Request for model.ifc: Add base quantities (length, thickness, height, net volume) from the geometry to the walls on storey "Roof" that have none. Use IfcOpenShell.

First a look at what the model holds.

```python
import ifcopenshell
import ifcopenshell.util.element
import ifcopenshell.util.unit

model = ifcopenshell.open("model.ifc")
print(model.schema)
for unit_type in ("LENGTHUNIT", "AREAUNIT", "VOLUMEUNIT"):
    print(unit_type, ifcopenshell.util.unit.calculate_unit_scale(model, unit_type))
storey = next(s for s in model.by_type("IfcBuildingStorey") if s.Name == "Roof")
walls = [e for e in ifcopenshell.util.element.get_decomposition(storey) if e.is_a("IfcWall")]
for e in sorted(walls, key=lambda e: e.id()):
    print(e.id(), e.is_a(), e.Name, list(ifcopenshell.util.element.get_psets(e, qtos_only=True)), sep=" | ")
```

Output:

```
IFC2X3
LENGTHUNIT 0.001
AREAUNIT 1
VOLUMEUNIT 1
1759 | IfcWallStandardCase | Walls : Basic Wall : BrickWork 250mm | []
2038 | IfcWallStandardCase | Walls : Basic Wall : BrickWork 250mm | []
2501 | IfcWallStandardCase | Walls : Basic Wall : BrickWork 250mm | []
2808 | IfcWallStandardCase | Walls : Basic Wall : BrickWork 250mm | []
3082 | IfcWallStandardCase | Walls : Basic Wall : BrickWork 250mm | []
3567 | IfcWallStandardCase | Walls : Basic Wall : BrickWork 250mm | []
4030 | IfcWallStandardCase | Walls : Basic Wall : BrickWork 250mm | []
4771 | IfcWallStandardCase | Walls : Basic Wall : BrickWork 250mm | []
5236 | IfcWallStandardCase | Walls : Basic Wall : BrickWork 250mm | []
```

```python
import ifcopenshell
import ifcopenshell.api.pset
import ifcopenshell.geom
import ifcopenshell.util.element
import ifcopenshell.util.shape
import ifcopenshell.util.unit

model = ifcopenshell.open("model.ifc")
unit_scale = ifcopenshell.util.unit.calculate_unit_scale(model)
volume_scale = ifcopenshell.util.unit.calculate_unit_scale(model, "VOLUMEUNIT")
settings = ifcopenshell.geom.settings()

storey = next(s for s in model.by_type("IfcBuildingStorey") if s.Name == "Roof")
walls = [e for e in ifcopenshell.util.element.get_decomposition(storey) if e.is_a("IfcWall")]

for e in sorted(walls, key=lambda e: e.id()):
    if ifcopenshell.util.element.get_psets(e, qtos_only=True, should_inherit=False):
        continue
    # Geometry comes back in metres, in the element's own axes.
    shape = ifcopenshell.geom.create_shape(settings, e)
    values = {
        "Length": ifcopenshell.util.shape.get_x(shape.geometry) / unit_scale,
        "Width": ifcopenshell.util.shape.get_y(shape.geometry) / unit_scale,
        "Height": ifcopenshell.util.shape.get_z(shape.geometry) / unit_scale,
        "NetVolume": ifcopenshell.util.shape.get_volume(shape.geometry) / volume_scale,
    }
    qto = ifcopenshell.api.pset.add_qto(model, product=e, name="BaseQuantities")
    ifcopenshell.api.pset.edit_qto(model, qto=qto, properties=values)
    print(e.id(), {k: round(v, 3) for k, v in values.items()})

model.write("model_updated.ifc")
```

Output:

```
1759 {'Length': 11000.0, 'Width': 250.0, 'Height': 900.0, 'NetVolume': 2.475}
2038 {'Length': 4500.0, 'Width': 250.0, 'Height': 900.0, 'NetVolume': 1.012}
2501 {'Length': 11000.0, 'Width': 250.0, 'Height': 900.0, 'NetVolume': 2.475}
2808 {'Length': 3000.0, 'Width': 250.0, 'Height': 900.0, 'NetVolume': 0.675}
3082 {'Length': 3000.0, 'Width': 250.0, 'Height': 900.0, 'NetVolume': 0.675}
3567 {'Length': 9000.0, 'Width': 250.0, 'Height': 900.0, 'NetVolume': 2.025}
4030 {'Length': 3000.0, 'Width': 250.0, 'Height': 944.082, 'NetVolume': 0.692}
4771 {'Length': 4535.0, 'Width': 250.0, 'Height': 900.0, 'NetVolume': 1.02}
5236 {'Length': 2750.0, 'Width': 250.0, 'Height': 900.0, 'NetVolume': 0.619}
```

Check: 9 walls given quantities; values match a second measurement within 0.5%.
